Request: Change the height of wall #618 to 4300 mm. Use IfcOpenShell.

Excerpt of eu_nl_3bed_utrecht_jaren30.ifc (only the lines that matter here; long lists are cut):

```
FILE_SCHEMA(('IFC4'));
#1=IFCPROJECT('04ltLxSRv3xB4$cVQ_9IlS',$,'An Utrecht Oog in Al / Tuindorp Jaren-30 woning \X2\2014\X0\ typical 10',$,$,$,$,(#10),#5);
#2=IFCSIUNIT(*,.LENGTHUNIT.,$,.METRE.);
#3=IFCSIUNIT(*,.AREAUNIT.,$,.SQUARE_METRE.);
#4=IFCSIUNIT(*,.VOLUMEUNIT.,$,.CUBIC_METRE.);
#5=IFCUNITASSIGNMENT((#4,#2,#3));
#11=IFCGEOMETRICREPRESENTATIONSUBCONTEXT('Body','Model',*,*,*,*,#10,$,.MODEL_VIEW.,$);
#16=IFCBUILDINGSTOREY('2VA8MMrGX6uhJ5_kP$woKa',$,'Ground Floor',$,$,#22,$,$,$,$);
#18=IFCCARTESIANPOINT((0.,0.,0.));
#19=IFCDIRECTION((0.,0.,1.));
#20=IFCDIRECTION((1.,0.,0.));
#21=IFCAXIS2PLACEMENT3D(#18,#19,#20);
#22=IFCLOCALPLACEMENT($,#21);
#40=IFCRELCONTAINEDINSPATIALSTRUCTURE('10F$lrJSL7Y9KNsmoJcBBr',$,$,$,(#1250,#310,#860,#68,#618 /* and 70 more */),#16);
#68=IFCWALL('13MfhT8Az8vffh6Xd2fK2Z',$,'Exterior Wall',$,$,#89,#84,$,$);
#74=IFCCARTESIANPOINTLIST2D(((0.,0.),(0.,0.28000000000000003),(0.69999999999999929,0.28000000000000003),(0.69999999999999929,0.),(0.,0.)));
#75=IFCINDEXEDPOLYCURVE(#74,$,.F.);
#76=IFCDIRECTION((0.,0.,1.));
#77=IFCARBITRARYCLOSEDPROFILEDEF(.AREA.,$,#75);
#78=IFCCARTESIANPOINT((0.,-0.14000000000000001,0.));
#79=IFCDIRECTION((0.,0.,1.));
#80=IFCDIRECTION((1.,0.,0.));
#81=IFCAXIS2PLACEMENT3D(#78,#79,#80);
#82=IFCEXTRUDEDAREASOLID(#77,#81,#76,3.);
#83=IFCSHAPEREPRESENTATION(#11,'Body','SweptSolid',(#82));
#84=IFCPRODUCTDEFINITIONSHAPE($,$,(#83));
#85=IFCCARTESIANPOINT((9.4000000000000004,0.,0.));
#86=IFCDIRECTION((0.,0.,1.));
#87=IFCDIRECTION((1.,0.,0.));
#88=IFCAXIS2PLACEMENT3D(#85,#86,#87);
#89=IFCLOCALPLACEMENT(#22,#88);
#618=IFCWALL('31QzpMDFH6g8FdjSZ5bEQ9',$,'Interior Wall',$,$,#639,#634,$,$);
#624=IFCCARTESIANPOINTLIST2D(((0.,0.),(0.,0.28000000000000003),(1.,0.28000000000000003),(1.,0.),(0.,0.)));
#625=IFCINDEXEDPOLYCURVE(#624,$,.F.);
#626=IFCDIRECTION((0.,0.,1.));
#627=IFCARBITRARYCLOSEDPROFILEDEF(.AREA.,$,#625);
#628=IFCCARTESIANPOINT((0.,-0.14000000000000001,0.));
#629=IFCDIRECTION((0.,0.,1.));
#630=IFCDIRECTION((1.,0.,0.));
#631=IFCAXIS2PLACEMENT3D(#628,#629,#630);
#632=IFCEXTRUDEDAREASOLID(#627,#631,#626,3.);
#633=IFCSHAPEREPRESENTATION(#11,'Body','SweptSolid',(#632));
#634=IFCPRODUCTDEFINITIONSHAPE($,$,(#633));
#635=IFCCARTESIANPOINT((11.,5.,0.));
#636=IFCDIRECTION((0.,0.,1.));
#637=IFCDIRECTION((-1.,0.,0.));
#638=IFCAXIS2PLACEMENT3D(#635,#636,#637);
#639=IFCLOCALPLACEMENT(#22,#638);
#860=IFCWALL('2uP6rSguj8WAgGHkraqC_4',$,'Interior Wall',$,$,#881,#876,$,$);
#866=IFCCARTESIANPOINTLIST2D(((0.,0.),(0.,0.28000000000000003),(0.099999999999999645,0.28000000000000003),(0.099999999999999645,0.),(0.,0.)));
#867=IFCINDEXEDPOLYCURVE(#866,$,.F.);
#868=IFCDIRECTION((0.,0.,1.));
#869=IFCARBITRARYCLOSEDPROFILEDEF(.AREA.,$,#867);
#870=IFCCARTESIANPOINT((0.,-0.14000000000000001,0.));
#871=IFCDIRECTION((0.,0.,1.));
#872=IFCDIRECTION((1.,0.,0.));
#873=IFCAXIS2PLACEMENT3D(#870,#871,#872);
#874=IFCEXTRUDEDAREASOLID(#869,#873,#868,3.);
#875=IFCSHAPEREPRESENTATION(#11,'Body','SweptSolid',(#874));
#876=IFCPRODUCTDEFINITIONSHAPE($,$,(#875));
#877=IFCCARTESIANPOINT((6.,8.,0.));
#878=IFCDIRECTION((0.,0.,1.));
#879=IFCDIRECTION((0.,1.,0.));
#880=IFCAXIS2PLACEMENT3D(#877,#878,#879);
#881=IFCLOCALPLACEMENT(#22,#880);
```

```python
import ifcopenshell
import ifcopenshell.geom
import ifcopenshell.util.representation
import ifcopenshell.util.shape
import ifcopenshell.util.unit

model = ifcopenshell.open("eu_nl_3bed_utrecht_jaren30.ifc")
unit_scale = ifcopenshell.util.unit.calculate_unit_scale(model)
settings = ifcopenshell.geom.settings()


def volume(element):
    """Net volume in cubic metres, openings subtracted."""
    shape = ifcopenshell.geom.create_shape(settings, element)
    return ifcopenshell.util.shape.get_volume(shape.geometry)


wall = model.by_id(618)
before = volume(wall)

body = ifcopenshell.util.representation.get_representation(wall, "Model", "Body")
solid = body.Items[0]
old_height = solid.Depth
solid.Depth = 4.3 / unit_scale
after = volume(wall)

print(f"height {old_height:g} -> {solid.Depth:g}, volume {before:.3f} -> {after:.3f} m3")

model.write("eu_nl_3bed_utrecht_jaren30_updated.ifc")
```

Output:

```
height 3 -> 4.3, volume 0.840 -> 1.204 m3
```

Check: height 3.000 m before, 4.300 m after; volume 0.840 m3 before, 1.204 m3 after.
